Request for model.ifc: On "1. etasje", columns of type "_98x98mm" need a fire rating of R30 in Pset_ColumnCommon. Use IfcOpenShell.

First a look at what the model holds.

```python
import ifcopenshell
import ifcopenshell.util.element

model = ifcopenshell.open("model.ifc")
print(model.schema)
storey = next(s for s in model.by_type("IfcBuildingStorey") if s.Name == "1. etasje")
columns = [e for e in ifcopenshell.util.element.get_decomposition(storey) if e.is_a("IfcColumn")]
seen = {}
for e in columns:
    element_type = ifcopenshell.util.element.get_type(e)
    key = (element_type.Name if element_type != e and element_type else None, ifcopenshell.util.element.get_pset(e, "Pset_ColumnCommon", "FireRating"))
    seen[key] = seen.get(key, 0) + 1
for (name, value), count in sorted(seen.items(), key=str):
    print(count, "x", name, "|", value)
```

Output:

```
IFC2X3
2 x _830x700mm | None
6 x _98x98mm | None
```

```python
import ifcopenshell
import ifcopenshell.api.pset
import ifcopenshell.util.element

model = ifcopenshell.open("model.ifc")

storey = next(s for s in model.by_type("IfcBuildingStorey") if s.Name == "1. etasje")
columns = [e for e in ifcopenshell.util.element.get_decomposition(storey) if e.is_a("IfcColumn")]

count = 0
for e in columns:
    element_type = ifcopenshell.util.element.get_type(e)
    if element_type in (None, e) or element_type.Name != "_98x98mm":
        continue
    # add_pset returns the element's existing set when there is one.
    pset = ifcopenshell.api.pset.add_pset(model, product=e, name="Pset_ColumnCommon")
    ifcopenshell.api.pset.edit_pset(model, pset=pset, properties={"FireRating": "R30"})
    count += 1

print(count, "columns updated")

model.write("model-out.ifc")
```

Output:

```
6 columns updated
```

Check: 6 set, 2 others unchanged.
